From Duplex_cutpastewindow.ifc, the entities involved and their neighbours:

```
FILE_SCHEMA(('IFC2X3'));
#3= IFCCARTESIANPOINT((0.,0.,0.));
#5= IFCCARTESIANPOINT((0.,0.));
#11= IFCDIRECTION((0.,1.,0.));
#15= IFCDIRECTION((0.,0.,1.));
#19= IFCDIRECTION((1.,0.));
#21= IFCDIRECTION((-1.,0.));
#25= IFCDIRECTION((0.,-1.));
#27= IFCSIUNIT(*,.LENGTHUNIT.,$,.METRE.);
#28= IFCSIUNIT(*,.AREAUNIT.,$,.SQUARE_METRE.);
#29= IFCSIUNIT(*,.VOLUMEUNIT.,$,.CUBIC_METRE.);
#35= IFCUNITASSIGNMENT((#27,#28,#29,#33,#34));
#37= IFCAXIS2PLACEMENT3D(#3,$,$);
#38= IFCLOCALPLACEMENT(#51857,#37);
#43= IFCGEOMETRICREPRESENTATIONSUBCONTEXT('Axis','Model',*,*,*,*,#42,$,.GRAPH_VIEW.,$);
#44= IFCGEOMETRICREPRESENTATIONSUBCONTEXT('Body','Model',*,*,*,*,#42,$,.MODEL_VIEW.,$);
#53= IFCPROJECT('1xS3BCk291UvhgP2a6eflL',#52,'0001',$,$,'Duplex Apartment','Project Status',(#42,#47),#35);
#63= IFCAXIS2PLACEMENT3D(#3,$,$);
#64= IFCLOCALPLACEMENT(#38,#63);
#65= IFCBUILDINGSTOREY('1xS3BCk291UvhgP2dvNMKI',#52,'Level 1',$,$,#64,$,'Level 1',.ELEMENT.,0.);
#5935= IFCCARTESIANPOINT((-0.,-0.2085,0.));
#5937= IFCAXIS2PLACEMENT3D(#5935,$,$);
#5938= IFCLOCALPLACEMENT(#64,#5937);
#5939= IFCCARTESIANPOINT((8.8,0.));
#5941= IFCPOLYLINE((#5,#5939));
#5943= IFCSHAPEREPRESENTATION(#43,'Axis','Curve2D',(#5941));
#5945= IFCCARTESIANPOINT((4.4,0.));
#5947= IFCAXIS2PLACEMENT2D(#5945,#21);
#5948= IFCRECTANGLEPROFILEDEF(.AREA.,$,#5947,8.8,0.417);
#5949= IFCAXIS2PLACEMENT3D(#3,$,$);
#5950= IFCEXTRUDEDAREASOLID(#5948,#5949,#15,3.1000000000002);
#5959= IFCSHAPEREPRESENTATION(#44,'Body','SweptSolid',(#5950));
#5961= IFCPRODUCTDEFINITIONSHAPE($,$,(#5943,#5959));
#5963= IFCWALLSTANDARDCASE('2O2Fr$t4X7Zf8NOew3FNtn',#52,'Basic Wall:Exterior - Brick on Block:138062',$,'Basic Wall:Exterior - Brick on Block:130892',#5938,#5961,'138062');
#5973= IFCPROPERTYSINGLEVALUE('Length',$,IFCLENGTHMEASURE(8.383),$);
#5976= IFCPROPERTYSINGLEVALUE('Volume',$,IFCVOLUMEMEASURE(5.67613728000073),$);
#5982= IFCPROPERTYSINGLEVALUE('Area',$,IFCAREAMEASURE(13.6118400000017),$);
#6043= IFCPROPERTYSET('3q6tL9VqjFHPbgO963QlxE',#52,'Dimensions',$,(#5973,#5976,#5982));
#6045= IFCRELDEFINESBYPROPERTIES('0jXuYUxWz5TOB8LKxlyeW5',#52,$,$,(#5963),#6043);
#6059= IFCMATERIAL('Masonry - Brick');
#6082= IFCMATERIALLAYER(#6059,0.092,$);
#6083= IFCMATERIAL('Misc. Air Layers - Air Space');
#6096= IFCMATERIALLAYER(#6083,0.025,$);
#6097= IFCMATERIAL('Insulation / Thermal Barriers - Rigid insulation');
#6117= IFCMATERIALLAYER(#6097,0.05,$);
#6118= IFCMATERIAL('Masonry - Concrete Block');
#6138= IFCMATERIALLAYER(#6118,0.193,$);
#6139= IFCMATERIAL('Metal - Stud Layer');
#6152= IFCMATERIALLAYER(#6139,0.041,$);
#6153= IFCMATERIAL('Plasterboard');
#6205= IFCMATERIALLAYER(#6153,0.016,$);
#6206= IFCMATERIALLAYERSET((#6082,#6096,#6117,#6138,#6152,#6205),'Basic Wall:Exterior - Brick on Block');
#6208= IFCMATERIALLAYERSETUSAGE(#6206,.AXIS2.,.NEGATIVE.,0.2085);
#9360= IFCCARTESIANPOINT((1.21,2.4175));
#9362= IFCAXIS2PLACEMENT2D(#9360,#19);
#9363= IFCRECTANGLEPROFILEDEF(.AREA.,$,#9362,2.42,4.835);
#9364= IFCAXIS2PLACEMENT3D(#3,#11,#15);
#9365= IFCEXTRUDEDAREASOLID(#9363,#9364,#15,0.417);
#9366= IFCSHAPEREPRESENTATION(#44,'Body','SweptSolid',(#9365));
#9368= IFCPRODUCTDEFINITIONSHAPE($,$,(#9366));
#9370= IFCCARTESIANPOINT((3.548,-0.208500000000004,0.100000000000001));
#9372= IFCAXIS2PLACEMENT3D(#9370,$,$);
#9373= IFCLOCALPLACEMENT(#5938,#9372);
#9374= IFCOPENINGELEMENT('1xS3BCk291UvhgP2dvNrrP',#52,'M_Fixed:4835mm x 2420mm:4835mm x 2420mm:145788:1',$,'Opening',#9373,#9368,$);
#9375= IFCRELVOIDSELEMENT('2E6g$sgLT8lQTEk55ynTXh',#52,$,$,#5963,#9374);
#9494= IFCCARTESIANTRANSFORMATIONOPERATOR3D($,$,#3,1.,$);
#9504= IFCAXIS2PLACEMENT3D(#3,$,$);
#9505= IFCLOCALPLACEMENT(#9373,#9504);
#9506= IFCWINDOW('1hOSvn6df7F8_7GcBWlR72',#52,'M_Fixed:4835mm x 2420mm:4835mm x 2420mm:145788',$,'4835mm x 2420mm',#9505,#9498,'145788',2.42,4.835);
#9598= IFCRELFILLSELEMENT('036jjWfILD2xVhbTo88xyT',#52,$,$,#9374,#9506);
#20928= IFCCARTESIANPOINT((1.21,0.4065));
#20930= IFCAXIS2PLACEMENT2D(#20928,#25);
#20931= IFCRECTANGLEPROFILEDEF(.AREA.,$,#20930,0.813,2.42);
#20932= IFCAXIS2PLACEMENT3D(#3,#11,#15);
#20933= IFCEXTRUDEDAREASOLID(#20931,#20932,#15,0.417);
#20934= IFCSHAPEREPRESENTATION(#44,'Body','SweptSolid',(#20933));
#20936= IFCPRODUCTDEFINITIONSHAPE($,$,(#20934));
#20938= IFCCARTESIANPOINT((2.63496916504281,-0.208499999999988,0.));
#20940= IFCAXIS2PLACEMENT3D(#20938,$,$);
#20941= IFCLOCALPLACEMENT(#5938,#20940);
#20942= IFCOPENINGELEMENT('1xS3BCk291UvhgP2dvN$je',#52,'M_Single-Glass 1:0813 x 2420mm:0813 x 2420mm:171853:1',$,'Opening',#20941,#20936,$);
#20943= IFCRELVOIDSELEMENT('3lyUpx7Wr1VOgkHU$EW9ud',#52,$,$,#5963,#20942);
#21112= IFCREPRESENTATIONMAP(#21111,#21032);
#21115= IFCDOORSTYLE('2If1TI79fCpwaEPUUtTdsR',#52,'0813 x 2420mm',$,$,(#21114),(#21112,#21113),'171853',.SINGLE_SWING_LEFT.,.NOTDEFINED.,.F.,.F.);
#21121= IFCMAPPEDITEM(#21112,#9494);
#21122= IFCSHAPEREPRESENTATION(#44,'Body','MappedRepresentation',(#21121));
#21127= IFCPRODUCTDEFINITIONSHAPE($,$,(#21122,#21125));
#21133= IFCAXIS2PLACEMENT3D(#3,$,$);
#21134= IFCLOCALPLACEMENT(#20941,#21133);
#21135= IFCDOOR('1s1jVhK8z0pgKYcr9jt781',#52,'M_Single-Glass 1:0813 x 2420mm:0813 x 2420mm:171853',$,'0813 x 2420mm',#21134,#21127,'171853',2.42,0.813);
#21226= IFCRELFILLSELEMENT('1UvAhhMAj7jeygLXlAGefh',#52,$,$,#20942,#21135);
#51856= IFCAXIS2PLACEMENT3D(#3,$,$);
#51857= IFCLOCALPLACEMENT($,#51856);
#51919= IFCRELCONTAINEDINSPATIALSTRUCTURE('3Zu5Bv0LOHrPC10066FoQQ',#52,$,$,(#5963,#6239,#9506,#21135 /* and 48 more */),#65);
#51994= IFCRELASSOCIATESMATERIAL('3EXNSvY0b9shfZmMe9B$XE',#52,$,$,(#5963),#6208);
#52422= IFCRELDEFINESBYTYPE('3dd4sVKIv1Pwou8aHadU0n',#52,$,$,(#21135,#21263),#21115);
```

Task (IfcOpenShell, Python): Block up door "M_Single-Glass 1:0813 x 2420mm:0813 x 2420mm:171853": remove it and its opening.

```python
import ifcopenshell
import ifcopenshell.api.feature
import ifcopenshell.api.pset
import ifcopenshell.api.root
import ifcopenshell.geom
import ifcopenshell.util.element
import ifcopenshell.util.shape
import ifcopenshell.util.unit

model = ifcopenshell.open("Duplex_cutpastewindow.ifc")
area_scale = ifcopenshell.util.unit.calculate_unit_scale(model, "AREAUNIT")
volume_scale = ifcopenshell.util.unit.calculate_unit_scale(model, "VOLUMEUNIT")
settings = ifcopenshell.geom.settings()


def volume(element):
    """Net volume in cubic metres, openings subtracted."""
    shape = ifcopenshell.geom.create_shape(settings, element)
    return ifcopenshell.util.shape.get_volume(shape.geometry)


door = model.by_guid("1s1jVhK8z0pgKYcr9jt781")
opening = door.FillsVoids[0].RelatingOpeningElement
wall = opening.VoidsElements[0].RelatingBuildingElement
before = volume(wall)

ifcopenshell.api.root.remove_product(model, product=door)
ifcopenshell.api.feature.remove_feature(model, feature=opening)

after = volume(wall)
thickness = 0.417  # wall thickness in metres

# Update the wall's stored quantities.
pset = model.by_id(ifcopenshell.util.element.get_pset(wall, "Dimensions", should_inherit=False)["id"])
ifcopenshell.api.pset.edit_pset(model, pset=pset, properties={
    "Volume": model.create_entity("IfcVolumeMeasure", after / volume_scale),
    "Area": model.create_entity("IfcAreaMeasure", after / thickness / area_scale),
})

print(f"wall volume {before:.3f} -> {after:.3f} m3")

model.write("Duplex_cutpastewindow_updated.ifc")
```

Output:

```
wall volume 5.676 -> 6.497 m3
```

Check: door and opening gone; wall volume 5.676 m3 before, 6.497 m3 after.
